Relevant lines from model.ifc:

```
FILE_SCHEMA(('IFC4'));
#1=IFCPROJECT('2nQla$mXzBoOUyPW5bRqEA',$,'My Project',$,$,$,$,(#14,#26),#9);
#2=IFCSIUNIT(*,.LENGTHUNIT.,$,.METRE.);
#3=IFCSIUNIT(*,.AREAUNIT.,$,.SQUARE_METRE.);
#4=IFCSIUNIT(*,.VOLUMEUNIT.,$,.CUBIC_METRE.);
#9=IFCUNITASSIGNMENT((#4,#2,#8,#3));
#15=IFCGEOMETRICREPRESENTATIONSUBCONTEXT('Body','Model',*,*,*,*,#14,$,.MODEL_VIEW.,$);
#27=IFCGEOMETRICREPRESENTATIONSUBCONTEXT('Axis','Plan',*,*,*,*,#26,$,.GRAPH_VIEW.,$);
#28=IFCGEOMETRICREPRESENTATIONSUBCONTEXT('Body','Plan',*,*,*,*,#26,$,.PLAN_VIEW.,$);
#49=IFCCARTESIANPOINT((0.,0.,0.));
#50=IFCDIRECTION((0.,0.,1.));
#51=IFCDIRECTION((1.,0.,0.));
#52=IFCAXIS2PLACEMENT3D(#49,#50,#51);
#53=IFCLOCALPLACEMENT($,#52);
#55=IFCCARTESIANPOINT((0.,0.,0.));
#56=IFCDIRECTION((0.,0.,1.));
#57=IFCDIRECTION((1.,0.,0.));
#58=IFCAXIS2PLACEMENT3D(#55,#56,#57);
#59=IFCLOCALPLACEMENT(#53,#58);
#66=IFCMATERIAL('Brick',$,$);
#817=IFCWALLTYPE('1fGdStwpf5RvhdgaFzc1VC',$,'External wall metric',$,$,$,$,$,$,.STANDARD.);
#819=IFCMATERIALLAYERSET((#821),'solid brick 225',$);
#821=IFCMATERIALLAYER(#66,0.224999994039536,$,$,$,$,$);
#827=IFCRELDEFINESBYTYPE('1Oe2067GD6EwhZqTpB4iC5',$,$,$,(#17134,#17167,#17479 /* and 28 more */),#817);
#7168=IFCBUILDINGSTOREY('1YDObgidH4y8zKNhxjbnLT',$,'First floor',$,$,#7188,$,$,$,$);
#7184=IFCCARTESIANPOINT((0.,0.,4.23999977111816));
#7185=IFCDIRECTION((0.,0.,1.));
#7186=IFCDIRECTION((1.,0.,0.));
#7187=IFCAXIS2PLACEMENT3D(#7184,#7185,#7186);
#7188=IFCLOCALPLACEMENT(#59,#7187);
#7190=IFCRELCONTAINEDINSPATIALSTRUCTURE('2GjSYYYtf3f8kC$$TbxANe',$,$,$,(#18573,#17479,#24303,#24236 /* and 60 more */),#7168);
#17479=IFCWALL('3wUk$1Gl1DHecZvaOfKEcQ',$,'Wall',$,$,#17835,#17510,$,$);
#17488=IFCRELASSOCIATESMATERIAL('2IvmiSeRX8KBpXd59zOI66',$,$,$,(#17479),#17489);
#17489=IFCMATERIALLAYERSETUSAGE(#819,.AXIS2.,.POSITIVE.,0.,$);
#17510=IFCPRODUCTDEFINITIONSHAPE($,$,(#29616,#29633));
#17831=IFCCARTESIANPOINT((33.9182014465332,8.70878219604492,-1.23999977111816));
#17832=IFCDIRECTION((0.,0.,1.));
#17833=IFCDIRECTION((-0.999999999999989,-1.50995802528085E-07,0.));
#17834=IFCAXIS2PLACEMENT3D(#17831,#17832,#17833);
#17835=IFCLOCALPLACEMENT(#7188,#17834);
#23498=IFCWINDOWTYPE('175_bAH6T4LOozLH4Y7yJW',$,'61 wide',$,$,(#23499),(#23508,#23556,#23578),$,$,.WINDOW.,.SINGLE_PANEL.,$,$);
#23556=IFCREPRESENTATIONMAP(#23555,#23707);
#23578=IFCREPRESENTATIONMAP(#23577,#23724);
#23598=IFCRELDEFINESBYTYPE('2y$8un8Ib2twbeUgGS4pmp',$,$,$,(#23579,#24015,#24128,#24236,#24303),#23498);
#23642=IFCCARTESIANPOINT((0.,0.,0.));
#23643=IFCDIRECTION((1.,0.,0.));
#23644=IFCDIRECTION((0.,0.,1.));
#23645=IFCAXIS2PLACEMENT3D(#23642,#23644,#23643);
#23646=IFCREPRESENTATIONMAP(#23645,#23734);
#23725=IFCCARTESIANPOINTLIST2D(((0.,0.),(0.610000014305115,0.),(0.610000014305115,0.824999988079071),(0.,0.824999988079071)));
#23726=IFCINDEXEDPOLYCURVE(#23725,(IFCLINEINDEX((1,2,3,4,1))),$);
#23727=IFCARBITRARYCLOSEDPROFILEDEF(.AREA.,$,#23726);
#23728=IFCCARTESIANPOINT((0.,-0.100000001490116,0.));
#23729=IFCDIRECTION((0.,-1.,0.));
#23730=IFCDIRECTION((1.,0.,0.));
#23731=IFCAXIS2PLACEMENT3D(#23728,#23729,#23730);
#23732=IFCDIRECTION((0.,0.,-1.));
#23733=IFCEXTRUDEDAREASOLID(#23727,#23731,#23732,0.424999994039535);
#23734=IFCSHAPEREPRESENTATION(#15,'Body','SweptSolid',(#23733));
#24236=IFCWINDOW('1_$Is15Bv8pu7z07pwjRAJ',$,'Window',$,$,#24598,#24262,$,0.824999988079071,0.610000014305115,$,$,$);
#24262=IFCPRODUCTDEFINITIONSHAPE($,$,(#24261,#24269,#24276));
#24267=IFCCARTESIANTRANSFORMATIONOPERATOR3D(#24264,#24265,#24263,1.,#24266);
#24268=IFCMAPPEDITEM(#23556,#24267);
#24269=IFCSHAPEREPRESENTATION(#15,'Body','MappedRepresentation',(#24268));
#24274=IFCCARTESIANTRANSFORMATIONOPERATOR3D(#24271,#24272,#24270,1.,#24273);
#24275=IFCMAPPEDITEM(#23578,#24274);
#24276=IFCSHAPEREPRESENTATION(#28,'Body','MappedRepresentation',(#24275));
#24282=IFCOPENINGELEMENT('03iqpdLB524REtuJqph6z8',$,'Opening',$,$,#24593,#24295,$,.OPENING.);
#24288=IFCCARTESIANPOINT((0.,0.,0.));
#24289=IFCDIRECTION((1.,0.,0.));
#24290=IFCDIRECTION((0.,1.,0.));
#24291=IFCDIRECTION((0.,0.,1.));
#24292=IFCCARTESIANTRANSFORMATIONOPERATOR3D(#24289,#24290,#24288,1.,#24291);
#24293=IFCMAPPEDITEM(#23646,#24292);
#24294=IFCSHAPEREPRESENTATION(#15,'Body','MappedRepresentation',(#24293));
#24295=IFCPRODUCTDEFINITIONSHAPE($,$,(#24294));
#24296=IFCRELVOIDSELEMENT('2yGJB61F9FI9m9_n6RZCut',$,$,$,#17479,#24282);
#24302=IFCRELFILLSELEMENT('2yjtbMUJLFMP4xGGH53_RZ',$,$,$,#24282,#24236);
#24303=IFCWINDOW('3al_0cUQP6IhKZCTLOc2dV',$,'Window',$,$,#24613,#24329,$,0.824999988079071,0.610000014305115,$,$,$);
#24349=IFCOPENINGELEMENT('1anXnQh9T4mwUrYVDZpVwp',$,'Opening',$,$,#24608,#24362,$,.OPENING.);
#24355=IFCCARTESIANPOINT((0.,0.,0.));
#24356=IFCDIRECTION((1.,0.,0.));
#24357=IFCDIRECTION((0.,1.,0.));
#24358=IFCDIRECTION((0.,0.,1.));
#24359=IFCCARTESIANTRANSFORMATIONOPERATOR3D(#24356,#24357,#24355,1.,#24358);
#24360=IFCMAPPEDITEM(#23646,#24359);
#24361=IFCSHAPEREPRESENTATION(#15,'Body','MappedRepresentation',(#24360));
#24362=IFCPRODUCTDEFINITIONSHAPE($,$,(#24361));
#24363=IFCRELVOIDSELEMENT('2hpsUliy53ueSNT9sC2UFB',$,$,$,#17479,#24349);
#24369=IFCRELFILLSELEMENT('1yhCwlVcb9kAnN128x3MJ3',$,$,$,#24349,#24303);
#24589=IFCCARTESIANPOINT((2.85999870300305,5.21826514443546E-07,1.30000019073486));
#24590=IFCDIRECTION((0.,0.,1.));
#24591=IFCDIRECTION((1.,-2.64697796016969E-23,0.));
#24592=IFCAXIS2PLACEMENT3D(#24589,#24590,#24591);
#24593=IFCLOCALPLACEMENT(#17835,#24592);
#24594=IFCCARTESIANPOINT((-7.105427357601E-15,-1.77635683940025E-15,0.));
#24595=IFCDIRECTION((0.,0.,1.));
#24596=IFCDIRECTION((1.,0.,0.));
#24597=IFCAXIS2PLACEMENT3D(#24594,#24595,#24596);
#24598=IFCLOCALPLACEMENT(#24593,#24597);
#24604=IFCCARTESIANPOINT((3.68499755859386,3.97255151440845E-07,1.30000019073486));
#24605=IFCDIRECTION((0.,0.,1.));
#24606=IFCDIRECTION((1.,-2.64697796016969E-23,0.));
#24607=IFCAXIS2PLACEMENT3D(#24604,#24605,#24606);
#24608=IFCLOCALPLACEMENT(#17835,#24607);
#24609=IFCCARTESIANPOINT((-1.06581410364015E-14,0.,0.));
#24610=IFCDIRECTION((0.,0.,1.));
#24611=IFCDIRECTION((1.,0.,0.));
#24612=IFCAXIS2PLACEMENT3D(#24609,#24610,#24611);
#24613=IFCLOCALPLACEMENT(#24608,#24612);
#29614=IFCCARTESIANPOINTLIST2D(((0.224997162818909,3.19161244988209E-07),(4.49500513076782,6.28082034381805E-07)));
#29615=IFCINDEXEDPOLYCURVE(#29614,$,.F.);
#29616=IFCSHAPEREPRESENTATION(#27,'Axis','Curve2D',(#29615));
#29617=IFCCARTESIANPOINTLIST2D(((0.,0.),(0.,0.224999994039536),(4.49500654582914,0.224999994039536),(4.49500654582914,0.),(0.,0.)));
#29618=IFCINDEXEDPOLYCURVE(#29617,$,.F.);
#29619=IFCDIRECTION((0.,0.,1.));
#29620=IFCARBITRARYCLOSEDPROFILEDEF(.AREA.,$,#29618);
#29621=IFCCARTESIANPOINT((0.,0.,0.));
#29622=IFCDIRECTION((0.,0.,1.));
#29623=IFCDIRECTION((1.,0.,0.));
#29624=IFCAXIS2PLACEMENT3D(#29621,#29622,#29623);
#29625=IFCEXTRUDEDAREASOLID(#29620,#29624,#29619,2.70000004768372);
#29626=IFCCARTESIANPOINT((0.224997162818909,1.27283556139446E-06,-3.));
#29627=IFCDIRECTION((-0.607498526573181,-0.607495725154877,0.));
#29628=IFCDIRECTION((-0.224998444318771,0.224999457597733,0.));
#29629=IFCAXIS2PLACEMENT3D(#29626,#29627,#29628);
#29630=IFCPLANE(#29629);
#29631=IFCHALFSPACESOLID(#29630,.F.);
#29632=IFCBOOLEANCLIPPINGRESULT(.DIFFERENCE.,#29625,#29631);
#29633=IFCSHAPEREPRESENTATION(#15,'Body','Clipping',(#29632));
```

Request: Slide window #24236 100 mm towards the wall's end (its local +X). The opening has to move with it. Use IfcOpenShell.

```python
import ifcopenshell
import ifcopenshell.api.geometry
import ifcopenshell.util.placement

model = ifcopenshell.open("model.ifc")

window = model.by_id(24236)
opening = window.FillsVoids[0].RelatingOpeningElement
wall = opening.VoidsElements[0].RelatingBuildingElement

wall_matrix = ifcopenshell.util.placement.get_local_placement(wall.ObjectPlacement)
shift = wall_matrix[:3, 0] * 0.1
before = ifcopenshell.util.placement.get_local_placement(window.ObjectPlacement)[:3, 3].copy()

# The window is placed relative to its opening, so it follows when the opening moves.
matrix = ifcopenshell.util.placement.get_local_placement(opening.ObjectPlacement)
matrix[:3, 3] += shift
ifcopenshell.api.geometry.edit_object_placement(
    model, product=opening, matrix=matrix, is_si=False, should_transform_children=True
)

after = ifcopenshell.util.placement.get_local_placement(window.ObjectPlacement)[:3, 3]
print("window moved by", (after - before).round(3) + 0.0)

model.write("model_v2.ifc")
```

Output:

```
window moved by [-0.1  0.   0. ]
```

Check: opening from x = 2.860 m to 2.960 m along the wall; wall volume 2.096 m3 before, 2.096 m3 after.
